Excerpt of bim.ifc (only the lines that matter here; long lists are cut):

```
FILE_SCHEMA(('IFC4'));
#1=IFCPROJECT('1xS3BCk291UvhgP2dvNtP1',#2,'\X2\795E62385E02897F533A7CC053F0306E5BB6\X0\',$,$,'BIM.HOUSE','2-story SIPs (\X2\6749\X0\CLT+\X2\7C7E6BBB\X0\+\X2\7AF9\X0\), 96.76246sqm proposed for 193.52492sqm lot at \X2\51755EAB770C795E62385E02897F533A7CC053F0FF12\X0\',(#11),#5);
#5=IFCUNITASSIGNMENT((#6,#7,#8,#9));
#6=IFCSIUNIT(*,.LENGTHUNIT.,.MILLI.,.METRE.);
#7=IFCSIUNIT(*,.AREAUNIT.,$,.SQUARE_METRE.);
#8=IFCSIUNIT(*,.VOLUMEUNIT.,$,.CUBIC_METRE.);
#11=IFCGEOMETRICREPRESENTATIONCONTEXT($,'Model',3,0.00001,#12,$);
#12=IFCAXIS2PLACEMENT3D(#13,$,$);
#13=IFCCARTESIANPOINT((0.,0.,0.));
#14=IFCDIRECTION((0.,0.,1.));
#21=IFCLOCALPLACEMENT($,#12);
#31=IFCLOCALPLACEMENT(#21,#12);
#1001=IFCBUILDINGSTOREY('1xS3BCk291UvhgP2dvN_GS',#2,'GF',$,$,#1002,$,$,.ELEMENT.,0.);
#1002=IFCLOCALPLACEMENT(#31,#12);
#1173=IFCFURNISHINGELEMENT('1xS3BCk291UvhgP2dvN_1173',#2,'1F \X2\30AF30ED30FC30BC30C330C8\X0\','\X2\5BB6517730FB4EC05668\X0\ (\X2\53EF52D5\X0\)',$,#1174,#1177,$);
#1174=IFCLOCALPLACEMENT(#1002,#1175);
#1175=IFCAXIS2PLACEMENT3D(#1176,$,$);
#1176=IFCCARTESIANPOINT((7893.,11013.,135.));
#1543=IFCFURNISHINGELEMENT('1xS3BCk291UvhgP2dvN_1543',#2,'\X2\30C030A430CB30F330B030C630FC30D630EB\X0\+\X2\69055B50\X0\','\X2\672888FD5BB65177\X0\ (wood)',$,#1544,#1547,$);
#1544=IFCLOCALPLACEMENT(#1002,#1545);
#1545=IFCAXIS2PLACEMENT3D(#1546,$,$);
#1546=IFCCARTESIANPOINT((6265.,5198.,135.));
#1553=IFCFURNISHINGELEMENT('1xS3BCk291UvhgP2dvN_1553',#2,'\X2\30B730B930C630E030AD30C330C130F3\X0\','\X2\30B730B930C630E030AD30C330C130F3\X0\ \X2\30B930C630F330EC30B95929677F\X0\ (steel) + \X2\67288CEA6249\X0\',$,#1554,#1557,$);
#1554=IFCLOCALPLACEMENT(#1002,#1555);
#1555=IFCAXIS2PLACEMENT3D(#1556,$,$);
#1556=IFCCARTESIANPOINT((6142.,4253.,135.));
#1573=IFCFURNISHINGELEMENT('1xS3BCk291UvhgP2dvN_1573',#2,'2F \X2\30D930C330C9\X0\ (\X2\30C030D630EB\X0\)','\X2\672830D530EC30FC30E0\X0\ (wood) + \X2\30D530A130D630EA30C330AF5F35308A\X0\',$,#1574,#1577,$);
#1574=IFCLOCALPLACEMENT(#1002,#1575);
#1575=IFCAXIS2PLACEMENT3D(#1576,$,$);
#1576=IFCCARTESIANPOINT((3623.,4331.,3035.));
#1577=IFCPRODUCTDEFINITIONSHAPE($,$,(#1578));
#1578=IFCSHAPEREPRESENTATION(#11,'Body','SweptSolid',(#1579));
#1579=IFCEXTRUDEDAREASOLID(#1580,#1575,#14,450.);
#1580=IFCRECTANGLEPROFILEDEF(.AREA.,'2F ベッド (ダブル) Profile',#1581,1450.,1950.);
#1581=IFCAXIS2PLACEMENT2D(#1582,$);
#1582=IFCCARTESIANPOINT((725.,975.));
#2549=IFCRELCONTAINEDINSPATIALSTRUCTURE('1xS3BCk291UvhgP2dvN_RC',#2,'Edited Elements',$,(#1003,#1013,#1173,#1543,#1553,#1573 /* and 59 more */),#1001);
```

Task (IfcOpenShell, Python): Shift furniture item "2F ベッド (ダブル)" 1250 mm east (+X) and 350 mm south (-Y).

```python
import ifcopenshell
import ifcopenshell.api.geometry
import ifcopenshell.util.placement
import ifcopenshell.util.unit

model = ifcopenshell.open("bim.ifc")
unit_scale = ifcopenshell.util.unit.calculate_unit_scale(model)

item = model.by_id(1573)
matrix = ifcopenshell.util.placement.get_local_placement(item.ObjectPlacement)
matrix[0, 3] += 1.25 / unit_scale
matrix[1, 3] -= 0.35 / unit_scale
ifcopenshell.api.geometry.edit_object_placement(model, product=item, matrix=matrix, is_si=False)

print(ifcopenshell.util.placement.get_local_placement(item.ObjectPlacement).round(3) + 0.0)

model.write("bim_v2.ifc")
```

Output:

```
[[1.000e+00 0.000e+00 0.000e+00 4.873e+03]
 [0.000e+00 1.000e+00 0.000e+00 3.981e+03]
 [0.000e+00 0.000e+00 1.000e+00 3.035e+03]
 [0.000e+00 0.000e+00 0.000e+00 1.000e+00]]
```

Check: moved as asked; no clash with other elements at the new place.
